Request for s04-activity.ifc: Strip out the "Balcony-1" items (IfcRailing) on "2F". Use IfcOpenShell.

First a look at what the model holds.

```python
import ifcopenshell
import ifcopenshell.util.element

model = ifcopenshell.open("s04-activity.ifc")
print(model.schema)
storey = next(s for s in model.by_type("IfcBuildingStorey") if s.Name == "2F")
railings = [e for e in ifcopenshell.util.element.get_decomposition(storey) if e.is_a("IfcRailing")]
seen = {}
for e in railings:
    element_type = ifcopenshell.util.element.get_type(e)
    name = element_type.Name if element_type not in (None, e) else None
    seen[name] = seen.get(name, 0) + 1
for name, count in sorted(seen.items(), key=str):
    print(count, "x", name)
```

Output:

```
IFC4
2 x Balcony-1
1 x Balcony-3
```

```python
import ifcopenshell
import ifcopenshell.api.root
import ifcopenshell.util.element

model = ifcopenshell.open("s04-activity.ifc")

storey = next(s for s in model.by_type("IfcBuildingStorey") if s.Name == "2F")
railings = [e for e in ifcopenshell.util.element.get_decomposition(storey) if e.is_a("IfcRailing")]
targets = [e for e in railings if (t := ifcopenshell.util.element.get_type(e)) not in (None, e) and t.Name == "Balcony-1"]

for e in targets:
    ifcopenshell.api.root.remove_product(model, product=e)
print(len(targets), "removed")

model.write("s04-activity_updated.ifc")
```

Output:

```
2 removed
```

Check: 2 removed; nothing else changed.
